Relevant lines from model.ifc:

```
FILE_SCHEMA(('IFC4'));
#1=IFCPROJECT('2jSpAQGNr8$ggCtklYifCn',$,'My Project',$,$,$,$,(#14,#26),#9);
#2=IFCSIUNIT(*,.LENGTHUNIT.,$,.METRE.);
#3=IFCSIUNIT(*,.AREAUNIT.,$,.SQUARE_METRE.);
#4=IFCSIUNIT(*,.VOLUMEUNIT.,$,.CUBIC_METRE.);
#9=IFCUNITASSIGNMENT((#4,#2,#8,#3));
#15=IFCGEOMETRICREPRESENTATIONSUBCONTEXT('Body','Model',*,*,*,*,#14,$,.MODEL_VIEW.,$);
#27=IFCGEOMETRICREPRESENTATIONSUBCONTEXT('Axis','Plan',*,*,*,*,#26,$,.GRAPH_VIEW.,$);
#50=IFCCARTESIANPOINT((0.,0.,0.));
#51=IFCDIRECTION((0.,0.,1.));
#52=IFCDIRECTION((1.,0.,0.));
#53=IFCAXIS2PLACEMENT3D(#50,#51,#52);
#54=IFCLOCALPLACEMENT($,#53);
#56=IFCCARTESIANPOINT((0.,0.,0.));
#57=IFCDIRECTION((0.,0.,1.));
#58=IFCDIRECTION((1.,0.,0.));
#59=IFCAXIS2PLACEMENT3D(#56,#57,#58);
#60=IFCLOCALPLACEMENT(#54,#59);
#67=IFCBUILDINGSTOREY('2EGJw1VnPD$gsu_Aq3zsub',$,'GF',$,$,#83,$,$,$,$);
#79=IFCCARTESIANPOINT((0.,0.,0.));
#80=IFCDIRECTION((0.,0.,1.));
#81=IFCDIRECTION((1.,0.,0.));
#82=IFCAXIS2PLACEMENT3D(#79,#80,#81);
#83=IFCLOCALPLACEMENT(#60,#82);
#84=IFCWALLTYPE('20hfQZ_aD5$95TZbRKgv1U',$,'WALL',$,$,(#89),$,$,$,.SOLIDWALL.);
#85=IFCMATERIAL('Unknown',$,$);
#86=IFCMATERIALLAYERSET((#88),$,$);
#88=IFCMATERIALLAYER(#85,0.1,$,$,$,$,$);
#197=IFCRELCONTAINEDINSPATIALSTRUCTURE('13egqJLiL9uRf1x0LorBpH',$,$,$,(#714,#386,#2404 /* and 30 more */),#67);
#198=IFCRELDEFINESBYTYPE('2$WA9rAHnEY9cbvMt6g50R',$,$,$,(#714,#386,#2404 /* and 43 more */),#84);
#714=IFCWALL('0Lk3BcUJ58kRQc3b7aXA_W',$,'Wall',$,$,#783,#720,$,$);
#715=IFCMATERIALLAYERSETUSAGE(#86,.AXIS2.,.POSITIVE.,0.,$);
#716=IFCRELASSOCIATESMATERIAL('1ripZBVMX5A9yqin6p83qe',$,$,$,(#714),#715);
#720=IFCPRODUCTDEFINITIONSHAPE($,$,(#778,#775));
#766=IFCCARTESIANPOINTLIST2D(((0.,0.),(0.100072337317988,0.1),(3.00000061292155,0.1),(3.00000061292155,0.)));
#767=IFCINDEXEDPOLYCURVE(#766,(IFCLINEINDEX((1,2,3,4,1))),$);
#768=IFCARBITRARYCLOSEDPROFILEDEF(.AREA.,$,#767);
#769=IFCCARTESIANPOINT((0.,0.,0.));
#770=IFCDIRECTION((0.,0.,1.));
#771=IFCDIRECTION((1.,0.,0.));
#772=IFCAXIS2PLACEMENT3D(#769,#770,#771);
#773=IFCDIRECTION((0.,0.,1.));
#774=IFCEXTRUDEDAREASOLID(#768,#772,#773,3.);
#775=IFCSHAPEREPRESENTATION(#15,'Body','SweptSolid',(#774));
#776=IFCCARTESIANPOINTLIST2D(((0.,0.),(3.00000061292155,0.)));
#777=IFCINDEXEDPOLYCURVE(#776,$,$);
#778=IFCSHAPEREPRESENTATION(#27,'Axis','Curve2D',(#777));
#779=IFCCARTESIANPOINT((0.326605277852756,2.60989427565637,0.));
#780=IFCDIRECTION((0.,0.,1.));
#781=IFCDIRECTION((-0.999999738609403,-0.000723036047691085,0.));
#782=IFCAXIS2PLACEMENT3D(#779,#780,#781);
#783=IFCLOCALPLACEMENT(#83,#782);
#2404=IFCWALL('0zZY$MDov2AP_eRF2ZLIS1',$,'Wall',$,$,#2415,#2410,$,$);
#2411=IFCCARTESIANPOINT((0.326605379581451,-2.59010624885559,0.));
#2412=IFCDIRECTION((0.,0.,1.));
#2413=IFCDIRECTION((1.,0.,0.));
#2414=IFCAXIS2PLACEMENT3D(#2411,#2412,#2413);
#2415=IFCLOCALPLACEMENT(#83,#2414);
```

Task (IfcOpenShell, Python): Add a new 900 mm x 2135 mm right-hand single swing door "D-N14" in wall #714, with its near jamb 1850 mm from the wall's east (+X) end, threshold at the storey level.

```python
import numpy as np
import ifcopenshell
import ifcopenshell.api.feature
import ifcopenshell.api.geometry
import ifcopenshell.api.root
import ifcopenshell.api.spatial
import ifcopenshell.geom
import ifcopenshell.util.element
import ifcopenshell.util.placement
import ifcopenshell.util.representation
import ifcopenshell.util.shape
import ifcopenshell.util.unit

model = ifcopenshell.open("model.ifc")
unit_scale = ifcopenshell.util.unit.calculate_unit_scale(model)
settings = ifcopenshell.geom.settings()


def volume(element):
    """Net volume in cubic metres, openings subtracted."""
    shape = ifcopenshell.geom.create_shape(settings, element)
    return ifcopenshell.util.shape.get_volume(shape.geometry)


wall = model.by_guid("0Lk3BcUJ58kRQc3b7aXA_W")
storey = ifcopenshell.util.element.get_container(wall, ifc_class="IfcBuildingStorey")
context = ifcopenshell.util.representation.get_context(model, "Model", "Body", "MODEL_VIEW")
before = volume(wall)

width, height, from_end, sill = 0.9, 2.135, 1.85, 0.0  # metres

# The wall runs along its own X axis, and the end named is its -X end.
wall_shape = ifcopenshell.geom.create_shape(settings, wall)
x, y, z = ifcopenshell.util.shape.get_vertices(wall_shape.geometry).T
start = x.min() + from_end
face, thickness = float(y.min()), float(y.max() - y.min())
wall_matrix = ifcopenshell.util.placement.get_local_placement(wall.ObjectPlacement)
level = ifcopenshell.util.placement.get_local_placement(storey.ObjectPlacement)[2, 3]


def in_wall(x, y):
    """Placement at x, y metres in the wall's axes, at sill height."""
    matrix = wall_matrix.copy()
    matrix[:, 3] = wall_matrix @ np.array([x / unit_scale, y / unit_scale, 0.0, 1.0])
    matrix[2, 3] = level + sill / unit_scale
    return matrix


# Opening: a box that overshoots both wall faces by 50 mm.
opening = ifcopenshell.api.root.create_entity(model, ifc_class="IfcOpeningElement", predefined_type="OPENING")
box = ifcopenshell.api.geometry.add_wall_representation(
    model, context=context, length=width, height=height, thickness=thickness + 0.1
)
ifcopenshell.api.geometry.assign_representation(model, product=opening, representation=box)
ifcopenshell.api.geometry.edit_object_placement(model, product=opening, matrix=in_wall(start, face - 0.05), is_si=False)
ifcopenshell.api.feature.add_feature(model, feature=opening, element=wall)

door = ifcopenshell.api.root.create_entity(model, ifc_class="IfcDoor", name="D-N14", predefined_type="DOOR")
door.OverallWidth, door.OverallHeight = width / unit_scale, height / unit_scale
door.OperationType = "SINGLE_SWING_RIGHT"
body = ifcopenshell.api.geometry.add_door_representation(
    model,
    context=context,
    overall_width=door.OverallWidth,
    overall_height=door.OverallHeight,
    operation_type="SINGLE_SWING_RIGHT",
    lining_properties={"LiningDepth": thickness / unit_scale, "ThresholdDepth": thickness / unit_scale},
)
ifcopenshell.api.geometry.assign_representation(model, product=door, representation=body)
ifcopenshell.api.spatial.assign_container(model, products=[door], relating_structure=storey)
ifcopenshell.api.feature.add_filling(model, opening=opening, element=door)

# The lining spans the wall, so the door starts at the wall face.
ifcopenshell.api.geometry.edit_object_placement(model, product=door, matrix=in_wall(start, face), is_si=False)

after = volume(wall)

print(f"wall volume {before:.3f} -> {after:.3f} m3")

model.write("model-out.ifc")
```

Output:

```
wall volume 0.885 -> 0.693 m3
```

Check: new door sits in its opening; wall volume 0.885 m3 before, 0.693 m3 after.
